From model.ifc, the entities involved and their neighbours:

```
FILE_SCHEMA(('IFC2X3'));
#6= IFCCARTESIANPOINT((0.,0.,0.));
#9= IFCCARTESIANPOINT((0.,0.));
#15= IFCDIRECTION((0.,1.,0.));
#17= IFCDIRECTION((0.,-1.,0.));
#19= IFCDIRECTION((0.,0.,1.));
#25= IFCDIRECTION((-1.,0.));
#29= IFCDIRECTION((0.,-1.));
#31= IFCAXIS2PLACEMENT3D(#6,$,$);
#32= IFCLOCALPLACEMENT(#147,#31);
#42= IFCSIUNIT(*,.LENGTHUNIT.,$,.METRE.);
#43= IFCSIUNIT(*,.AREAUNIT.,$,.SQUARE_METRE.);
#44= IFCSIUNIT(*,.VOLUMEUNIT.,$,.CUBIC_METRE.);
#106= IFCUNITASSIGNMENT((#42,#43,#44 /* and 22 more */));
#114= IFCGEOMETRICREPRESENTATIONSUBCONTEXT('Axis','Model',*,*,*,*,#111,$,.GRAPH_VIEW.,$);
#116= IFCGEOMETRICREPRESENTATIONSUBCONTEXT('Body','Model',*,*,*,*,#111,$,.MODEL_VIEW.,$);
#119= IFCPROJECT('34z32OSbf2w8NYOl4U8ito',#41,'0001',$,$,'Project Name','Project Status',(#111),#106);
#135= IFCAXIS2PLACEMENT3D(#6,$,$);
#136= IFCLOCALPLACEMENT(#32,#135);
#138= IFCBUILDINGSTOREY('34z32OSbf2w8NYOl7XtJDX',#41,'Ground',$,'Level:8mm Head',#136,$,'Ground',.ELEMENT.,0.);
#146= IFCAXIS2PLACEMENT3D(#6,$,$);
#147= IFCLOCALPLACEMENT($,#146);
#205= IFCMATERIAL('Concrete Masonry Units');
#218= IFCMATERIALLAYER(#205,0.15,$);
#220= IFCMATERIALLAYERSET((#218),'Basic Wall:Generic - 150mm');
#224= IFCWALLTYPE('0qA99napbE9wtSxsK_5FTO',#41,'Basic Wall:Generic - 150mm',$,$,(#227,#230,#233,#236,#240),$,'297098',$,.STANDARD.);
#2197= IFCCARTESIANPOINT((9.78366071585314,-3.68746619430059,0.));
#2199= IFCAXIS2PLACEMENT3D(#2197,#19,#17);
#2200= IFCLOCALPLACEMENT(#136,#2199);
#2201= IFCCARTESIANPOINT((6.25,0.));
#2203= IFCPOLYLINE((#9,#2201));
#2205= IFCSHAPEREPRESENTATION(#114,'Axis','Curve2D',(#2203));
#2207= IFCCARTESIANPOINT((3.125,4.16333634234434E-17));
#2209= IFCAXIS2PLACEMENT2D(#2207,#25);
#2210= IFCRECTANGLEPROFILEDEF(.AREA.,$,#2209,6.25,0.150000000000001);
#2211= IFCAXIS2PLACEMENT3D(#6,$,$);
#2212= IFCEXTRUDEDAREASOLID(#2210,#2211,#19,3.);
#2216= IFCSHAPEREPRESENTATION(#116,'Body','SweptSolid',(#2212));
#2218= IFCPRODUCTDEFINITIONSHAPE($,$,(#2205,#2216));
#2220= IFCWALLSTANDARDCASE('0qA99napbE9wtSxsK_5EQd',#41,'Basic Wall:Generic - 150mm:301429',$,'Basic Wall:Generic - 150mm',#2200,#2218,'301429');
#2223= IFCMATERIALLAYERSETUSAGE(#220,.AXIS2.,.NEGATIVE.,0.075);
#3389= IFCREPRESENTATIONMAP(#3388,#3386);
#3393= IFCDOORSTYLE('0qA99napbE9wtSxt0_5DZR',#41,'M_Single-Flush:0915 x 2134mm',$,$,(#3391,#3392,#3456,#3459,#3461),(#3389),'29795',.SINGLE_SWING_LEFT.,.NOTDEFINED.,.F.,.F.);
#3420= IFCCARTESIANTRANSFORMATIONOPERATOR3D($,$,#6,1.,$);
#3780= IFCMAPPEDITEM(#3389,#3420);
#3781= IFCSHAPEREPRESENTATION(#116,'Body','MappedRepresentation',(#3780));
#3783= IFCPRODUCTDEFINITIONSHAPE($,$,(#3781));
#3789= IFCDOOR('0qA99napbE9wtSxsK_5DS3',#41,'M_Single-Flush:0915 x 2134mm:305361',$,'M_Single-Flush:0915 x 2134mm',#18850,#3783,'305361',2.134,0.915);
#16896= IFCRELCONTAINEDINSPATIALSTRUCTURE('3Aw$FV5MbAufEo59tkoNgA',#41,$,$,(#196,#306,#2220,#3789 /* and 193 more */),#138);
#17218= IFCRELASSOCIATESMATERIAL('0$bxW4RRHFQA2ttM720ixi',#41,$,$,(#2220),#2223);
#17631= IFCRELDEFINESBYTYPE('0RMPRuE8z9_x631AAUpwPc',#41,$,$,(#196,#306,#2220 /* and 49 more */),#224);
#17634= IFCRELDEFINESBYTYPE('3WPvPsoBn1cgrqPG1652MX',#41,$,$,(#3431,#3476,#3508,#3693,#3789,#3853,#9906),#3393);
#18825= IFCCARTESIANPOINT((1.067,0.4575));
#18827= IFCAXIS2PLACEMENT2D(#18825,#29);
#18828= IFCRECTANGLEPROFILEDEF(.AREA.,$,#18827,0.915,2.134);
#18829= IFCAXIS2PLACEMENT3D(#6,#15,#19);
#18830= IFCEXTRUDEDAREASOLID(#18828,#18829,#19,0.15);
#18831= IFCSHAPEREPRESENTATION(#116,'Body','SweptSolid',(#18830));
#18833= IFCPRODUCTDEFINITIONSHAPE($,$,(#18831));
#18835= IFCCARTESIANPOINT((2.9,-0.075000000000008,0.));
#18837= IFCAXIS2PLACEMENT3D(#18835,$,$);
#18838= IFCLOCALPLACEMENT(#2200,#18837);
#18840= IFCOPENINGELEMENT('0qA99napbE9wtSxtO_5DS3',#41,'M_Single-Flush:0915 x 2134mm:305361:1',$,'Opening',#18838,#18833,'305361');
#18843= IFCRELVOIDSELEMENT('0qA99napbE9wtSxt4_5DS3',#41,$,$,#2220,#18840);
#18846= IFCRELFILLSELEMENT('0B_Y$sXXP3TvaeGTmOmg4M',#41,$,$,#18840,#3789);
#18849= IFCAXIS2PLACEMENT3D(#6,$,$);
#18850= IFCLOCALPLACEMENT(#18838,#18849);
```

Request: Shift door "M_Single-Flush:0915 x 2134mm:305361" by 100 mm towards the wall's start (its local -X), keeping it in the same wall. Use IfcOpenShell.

```python
import ifcopenshell
import ifcopenshell.api.geometry
import ifcopenshell.util.placement

model = ifcopenshell.open("model.ifc")

door = model.by_guid("0qA99napbE9wtSxsK_5DS3")
opening = door.FillsVoids[0].RelatingOpeningElement
wall = opening.VoidsElements[0].RelatingBuildingElement

wall_matrix = ifcopenshell.util.placement.get_local_placement(wall.ObjectPlacement)
shift = wall_matrix[:3, 0] * -0.1
before = ifcopenshell.util.placement.get_local_placement(door.ObjectPlacement)[:3, 3].copy()

# The door is placed relative to its opening, so it follows when the opening moves.
matrix = ifcopenshell.util.placement.get_local_placement(opening.ObjectPlacement)
matrix[:3, 3] += shift
ifcopenshell.api.geometry.edit_object_placement(
    model, product=opening, matrix=matrix, is_si=False, should_transform_children=True
)

after = ifcopenshell.util.placement.get_local_placement(door.ObjectPlacement)[:3, 3]
print("door moved by", (after - before).round(3) + 0.0)

model.write("model_updated.ifc")
```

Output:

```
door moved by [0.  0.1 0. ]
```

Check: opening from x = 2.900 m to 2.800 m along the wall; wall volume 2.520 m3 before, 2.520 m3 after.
